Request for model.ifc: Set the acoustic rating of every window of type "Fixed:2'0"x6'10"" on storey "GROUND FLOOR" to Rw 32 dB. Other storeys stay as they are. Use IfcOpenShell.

First a look at what the model holds.

```python
import ifcopenshell
import ifcopenshell.util.element

model = ifcopenshell.open("model.ifc")
print(model.schema)
storey = next(s for s in model.by_type("IfcBuildingStorey") if s.Name == "GROUND FLOOR")
windows = [e for e in ifcopenshell.util.element.get_decomposition(storey) if e.is_a("IfcWindow")]
seen = {}
for e in windows:
    element_type = ifcopenshell.util.element.get_type(e)
    key = (element_type.Name if element_type != e and element_type else None, ifcopenshell.util.element.get_pset(e, "Pset_WindowCommon", "AcousticRating"))
    seen[key] = seen.get(key, 0) + 1
for (name, value), count in sorted(seen.items(), key=str):
    print(count, "x", name, "|", value)
```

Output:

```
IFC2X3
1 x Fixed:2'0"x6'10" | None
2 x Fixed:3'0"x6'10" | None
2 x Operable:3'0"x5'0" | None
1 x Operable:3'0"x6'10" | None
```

```python
import ifcopenshell
import ifcopenshell.api.pset
import ifcopenshell.util.element

model = ifcopenshell.open("model.ifc")

storey = next(s for s in model.by_type("IfcBuildingStorey") if s.Name == "GROUND FLOOR")
windows = [e for e in ifcopenshell.util.element.get_decomposition(storey) if e.is_a("IfcWindow")]

count = 0
for e in windows:
    element_type = ifcopenshell.util.element.get_type(e)
    if element_type in (None, e) or element_type.Name != 'Fixed:2\'0"x6\'10"':
        continue
    # add_pset returns the element's existing set when there is one.
    pset = ifcopenshell.api.pset.add_pset(model, product=e, name="Pset_WindowCommon")
    ifcopenshell.api.pset.edit_pset(model, pset=pset, properties={"AcousticRating": "Rw 32 dB"})
    count += 1

print(count, "windows updated")

model.write("model_edited.ifc")
```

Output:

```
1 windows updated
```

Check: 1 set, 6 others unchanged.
